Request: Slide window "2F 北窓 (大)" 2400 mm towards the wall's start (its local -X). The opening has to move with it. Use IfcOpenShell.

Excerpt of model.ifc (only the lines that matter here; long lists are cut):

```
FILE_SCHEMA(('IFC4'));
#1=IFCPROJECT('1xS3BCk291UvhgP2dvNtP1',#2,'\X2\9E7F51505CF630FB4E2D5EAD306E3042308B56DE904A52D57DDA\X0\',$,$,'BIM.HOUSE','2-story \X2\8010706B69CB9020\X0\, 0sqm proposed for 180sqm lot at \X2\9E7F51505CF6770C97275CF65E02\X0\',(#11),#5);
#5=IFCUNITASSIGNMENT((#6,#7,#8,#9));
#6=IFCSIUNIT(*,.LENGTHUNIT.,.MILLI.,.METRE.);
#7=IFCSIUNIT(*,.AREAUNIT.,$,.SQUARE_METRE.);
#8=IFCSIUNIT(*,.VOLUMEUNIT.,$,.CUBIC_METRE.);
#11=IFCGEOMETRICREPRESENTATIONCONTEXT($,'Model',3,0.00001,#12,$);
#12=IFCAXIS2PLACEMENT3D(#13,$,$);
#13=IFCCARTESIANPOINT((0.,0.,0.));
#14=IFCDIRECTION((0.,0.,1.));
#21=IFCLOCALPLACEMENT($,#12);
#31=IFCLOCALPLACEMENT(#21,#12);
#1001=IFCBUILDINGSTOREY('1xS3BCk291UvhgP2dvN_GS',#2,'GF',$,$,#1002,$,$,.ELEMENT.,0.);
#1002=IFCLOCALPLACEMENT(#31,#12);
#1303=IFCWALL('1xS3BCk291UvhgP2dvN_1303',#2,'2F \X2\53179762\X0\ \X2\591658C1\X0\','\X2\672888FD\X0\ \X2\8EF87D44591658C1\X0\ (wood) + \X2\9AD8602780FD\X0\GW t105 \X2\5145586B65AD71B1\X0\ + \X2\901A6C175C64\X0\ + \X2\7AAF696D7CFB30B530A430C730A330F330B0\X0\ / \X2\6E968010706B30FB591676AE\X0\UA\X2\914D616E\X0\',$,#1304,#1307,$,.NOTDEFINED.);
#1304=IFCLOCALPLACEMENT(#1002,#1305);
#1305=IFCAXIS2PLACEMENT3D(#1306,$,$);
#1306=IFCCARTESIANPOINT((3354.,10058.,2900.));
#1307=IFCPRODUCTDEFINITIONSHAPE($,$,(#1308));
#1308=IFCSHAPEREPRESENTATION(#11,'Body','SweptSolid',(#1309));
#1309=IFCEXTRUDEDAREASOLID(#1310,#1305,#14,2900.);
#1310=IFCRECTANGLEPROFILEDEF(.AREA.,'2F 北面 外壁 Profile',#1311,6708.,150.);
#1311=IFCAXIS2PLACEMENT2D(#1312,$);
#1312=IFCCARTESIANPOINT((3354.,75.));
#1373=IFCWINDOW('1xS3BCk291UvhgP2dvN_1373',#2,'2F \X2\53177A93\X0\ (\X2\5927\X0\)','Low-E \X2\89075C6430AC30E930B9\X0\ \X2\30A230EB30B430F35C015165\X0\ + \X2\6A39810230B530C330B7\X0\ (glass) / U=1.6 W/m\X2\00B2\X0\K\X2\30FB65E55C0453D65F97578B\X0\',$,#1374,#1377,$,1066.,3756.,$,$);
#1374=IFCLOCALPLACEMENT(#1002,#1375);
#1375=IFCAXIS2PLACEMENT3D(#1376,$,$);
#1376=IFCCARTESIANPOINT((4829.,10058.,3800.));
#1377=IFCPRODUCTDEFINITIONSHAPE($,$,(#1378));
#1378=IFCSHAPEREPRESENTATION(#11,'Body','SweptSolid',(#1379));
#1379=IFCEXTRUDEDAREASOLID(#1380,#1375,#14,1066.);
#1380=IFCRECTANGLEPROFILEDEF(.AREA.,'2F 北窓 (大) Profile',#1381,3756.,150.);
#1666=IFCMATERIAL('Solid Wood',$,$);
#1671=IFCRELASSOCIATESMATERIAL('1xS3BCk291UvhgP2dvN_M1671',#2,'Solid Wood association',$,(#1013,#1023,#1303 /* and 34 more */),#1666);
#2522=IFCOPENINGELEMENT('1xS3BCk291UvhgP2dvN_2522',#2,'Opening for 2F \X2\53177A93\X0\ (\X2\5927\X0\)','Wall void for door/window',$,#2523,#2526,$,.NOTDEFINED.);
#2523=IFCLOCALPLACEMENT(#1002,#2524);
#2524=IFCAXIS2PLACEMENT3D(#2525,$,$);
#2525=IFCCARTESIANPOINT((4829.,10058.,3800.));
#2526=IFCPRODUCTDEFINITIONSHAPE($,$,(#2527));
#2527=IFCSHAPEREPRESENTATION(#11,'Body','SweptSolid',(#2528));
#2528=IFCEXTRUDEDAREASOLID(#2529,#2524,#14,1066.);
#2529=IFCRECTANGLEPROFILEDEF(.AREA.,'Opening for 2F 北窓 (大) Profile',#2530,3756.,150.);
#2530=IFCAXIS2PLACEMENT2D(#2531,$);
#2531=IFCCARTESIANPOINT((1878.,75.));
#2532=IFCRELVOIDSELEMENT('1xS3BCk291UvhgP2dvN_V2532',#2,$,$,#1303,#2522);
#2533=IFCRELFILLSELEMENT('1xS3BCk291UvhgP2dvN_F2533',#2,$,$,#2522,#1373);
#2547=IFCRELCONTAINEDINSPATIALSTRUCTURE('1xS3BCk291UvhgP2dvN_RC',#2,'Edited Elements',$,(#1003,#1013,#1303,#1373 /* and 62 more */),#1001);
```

```python
import ifcopenshell
import ifcopenshell.api.geometry
import ifcopenshell.util.placement

model = ifcopenshell.open("model.ifc")

window = model.by_id(1373)
opening = window.FillsVoids[0].RelatingOpeningElement
wall = opening.VoidsElements[0].RelatingBuildingElement

wall_matrix = ifcopenshell.util.placement.get_local_placement(wall.ObjectPlacement)
shift = wall_matrix[:3, 0] * -2400.0
before = ifcopenshell.util.placement.get_local_placement(window.ObjectPlacement)[:3, 3].copy()

# The window is not placed relative to its opening, so move both.
for product in (opening, window):
    matrix = ifcopenshell.util.placement.get_local_placement(product.ObjectPlacement)
    matrix[:3, 3] += shift
    ifcopenshell.api.geometry.edit_object_placement(model, product=product, matrix=matrix, is_si=False)

after = ifcopenshell.util.placement.get_local_placement(window.ObjectPlacement)[:3, 3]
print("window moved by", (after - before).round(3) + 0.0)

model.write("model_v2.ifc")
```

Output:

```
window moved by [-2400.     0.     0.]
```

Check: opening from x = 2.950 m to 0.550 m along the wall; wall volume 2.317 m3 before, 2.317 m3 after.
